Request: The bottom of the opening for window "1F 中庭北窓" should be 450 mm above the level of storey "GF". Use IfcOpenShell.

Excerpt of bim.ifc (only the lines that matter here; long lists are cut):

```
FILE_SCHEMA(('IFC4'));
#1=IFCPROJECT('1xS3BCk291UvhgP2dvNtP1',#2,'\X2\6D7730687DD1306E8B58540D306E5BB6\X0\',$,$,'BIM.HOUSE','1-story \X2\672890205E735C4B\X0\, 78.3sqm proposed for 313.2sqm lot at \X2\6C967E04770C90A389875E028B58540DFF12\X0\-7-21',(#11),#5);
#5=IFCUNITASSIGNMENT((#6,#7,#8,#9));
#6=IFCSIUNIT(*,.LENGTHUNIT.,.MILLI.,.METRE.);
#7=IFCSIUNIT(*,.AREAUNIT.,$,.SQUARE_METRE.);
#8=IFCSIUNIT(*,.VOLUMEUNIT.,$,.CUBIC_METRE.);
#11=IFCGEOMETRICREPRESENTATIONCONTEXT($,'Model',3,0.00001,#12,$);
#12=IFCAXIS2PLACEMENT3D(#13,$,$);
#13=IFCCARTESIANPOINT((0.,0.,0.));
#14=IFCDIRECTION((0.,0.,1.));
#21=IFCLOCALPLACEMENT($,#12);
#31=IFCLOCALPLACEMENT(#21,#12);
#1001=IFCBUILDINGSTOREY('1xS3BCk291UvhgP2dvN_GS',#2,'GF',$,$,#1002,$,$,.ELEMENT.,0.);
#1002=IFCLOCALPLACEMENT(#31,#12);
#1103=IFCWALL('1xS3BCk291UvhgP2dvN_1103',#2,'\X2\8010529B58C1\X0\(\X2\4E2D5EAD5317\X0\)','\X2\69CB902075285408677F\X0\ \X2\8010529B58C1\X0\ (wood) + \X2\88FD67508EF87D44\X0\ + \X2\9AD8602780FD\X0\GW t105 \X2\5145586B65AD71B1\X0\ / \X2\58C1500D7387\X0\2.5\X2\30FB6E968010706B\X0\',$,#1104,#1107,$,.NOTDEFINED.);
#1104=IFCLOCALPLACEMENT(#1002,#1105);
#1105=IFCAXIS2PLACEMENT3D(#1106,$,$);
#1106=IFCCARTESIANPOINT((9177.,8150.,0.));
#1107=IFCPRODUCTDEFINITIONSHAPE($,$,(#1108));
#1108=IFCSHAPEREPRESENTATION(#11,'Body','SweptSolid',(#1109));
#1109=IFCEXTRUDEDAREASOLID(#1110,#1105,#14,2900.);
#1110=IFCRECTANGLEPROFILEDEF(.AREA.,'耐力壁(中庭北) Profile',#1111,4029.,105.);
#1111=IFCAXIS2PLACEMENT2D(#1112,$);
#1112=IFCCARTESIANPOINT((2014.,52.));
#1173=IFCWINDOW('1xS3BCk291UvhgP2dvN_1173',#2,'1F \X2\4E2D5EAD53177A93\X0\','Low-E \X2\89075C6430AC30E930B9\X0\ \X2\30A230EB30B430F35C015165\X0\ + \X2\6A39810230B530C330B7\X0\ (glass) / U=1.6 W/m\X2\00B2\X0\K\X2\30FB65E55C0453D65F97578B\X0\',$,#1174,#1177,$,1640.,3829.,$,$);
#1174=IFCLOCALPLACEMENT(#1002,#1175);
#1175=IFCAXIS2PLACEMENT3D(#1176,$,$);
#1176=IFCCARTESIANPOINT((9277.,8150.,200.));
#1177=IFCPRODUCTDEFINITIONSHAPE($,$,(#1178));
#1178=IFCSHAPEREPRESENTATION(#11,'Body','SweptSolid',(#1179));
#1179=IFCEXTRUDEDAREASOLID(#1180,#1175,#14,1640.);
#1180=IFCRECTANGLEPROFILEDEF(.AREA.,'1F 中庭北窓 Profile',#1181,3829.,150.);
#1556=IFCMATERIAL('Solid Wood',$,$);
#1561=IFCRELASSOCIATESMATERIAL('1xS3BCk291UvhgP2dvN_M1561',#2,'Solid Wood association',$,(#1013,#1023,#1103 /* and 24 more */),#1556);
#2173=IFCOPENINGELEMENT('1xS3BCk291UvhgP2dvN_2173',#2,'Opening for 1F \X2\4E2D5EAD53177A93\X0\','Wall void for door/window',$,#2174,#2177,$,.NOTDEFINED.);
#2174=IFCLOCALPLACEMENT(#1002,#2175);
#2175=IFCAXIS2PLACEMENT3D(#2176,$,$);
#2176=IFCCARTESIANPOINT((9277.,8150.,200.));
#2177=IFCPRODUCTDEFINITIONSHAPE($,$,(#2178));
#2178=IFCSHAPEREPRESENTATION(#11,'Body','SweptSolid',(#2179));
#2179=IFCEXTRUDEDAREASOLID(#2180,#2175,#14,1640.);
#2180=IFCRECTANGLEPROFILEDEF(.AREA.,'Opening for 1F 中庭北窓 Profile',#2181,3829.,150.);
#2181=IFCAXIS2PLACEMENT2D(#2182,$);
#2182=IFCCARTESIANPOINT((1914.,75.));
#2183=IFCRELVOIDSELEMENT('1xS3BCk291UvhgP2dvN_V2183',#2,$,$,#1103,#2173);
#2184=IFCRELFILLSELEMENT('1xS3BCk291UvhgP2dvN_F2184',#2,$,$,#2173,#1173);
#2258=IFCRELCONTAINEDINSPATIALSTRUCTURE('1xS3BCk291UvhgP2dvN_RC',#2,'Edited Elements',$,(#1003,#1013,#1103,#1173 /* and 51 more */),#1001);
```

```python
import numpy as np
import ifcopenshell
import ifcopenshell.api.geometry
import ifcopenshell.geom
import ifcopenshell.util.element
import ifcopenshell.util.placement
import ifcopenshell.util.shape
import ifcopenshell.util.unit

model = ifcopenshell.open("bim.ifc")
unit_scale = ifcopenshell.util.unit.calculate_unit_scale(model)

window = model.by_guid("1xS3BCk291UvhgP2dvN_1173")
opening = window.FillsVoids[0].RelatingOpeningElement
storey = ifcopenshell.util.element.get_container(window, ifc_class="IfcBuildingStorey")
level = ifcopenshell.util.placement.get_local_placement(storey.ObjectPlacement)[2, 3]

# The opening's origin need not be at the sill, so measure its lowest point.
shape = ifcopenshell.geom.create_shape(ifcopenshell.geom.settings(), opening)
bottom = ifcopenshell.util.shape.get_shape_bottom_elevation(shape, shape.geometry) / unit_scale
dz = level + 0.45 / unit_scale - bottom

shift = np.array([0.0, 0.0, dz])
# The window is not placed relative to its opening, so move both.
for product in (opening, window):
    matrix = ifcopenshell.util.placement.get_local_placement(product.ObjectPlacement)
    matrix[:3, 3] += shift
    ifcopenshell.api.geometry.edit_object_placement(model, product=product, matrix=matrix, is_si=False)

print(f"moved by {dz * unit_scale:+.3f} m")

model.write("bim-out.ifc")
```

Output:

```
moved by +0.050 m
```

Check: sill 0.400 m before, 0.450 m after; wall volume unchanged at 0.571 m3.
